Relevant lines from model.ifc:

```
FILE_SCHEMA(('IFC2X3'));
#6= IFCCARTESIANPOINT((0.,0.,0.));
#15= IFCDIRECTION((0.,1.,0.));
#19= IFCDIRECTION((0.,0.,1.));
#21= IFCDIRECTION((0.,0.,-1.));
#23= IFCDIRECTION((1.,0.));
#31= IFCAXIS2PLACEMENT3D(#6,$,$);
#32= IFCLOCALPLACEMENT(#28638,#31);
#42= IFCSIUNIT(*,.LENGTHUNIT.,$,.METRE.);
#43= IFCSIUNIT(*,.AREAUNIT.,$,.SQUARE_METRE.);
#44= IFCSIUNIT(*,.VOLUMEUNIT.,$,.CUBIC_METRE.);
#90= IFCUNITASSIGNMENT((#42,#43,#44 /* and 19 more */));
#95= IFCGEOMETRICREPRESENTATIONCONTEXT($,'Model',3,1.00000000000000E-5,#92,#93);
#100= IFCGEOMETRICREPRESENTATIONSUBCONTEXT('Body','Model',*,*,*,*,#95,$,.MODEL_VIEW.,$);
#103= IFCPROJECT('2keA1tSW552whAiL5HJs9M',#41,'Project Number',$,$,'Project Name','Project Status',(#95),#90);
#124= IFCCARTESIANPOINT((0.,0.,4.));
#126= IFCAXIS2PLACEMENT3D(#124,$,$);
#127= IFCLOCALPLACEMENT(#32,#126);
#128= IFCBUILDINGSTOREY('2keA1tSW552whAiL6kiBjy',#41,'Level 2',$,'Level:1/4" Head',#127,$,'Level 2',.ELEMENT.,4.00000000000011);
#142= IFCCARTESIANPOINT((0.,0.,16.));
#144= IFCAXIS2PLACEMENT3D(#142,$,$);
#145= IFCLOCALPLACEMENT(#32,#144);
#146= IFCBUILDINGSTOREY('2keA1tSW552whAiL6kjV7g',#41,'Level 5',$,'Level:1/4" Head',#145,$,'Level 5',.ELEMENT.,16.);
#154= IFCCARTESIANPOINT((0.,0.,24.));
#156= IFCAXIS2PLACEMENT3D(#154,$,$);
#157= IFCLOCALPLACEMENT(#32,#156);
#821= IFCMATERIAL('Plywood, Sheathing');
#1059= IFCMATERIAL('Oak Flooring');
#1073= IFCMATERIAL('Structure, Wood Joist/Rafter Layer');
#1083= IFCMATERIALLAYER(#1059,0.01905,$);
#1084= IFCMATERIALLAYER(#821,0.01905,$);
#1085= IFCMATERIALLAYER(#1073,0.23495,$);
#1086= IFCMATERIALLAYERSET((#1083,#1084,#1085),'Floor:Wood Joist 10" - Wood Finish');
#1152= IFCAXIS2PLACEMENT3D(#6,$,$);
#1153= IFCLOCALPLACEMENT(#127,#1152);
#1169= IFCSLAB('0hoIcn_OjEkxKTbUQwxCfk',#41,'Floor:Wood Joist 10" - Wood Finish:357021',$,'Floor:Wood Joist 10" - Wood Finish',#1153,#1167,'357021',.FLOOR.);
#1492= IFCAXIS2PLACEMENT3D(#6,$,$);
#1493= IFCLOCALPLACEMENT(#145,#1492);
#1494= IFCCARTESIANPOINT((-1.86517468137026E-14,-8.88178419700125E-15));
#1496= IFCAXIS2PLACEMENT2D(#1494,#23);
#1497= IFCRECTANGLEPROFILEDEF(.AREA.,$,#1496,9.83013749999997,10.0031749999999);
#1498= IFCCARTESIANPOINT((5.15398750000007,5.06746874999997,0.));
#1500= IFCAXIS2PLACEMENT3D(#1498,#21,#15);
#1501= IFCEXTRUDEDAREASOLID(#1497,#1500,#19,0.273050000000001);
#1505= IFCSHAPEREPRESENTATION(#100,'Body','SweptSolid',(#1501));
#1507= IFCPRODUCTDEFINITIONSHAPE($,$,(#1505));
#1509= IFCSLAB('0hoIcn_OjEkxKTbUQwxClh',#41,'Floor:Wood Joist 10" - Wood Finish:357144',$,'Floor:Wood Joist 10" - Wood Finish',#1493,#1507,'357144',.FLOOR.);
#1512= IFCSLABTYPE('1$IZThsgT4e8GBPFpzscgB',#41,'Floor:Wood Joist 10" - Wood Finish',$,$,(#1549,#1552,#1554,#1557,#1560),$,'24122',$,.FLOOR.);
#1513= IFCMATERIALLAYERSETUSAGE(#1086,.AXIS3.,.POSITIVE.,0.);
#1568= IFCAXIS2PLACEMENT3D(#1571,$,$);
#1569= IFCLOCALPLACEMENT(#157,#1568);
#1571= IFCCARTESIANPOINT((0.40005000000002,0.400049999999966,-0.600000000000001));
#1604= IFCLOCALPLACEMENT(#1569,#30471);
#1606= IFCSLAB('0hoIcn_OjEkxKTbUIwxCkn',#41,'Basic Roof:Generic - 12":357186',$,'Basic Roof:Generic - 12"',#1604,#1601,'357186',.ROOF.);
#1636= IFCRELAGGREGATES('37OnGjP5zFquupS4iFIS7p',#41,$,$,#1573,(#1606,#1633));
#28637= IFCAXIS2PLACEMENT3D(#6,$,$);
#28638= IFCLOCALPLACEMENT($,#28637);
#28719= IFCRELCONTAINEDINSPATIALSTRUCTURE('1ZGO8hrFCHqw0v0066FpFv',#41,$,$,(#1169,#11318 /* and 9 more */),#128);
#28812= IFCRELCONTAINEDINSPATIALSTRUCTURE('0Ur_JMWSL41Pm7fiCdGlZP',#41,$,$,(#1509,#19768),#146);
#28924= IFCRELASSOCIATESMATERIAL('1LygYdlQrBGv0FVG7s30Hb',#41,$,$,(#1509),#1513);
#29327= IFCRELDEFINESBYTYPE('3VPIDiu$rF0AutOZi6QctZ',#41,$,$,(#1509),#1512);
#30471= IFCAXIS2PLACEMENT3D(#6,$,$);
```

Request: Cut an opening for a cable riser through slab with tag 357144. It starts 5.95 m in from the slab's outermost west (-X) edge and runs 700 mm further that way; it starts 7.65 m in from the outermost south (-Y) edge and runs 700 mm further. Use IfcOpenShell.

```python
import numpy as np
import ifcopenshell
import ifcopenshell.api.feature
import ifcopenshell.api.geometry
import ifcopenshell.api.root
import ifcopenshell.geom
import ifcopenshell.util.placement
import ifcopenshell.util.representation
import ifcopenshell.util.shape
import ifcopenshell.util.unit

model = ifcopenshell.open("model.ifc")
unit_scale = ifcopenshell.util.unit.calculate_unit_scale(model)
settings = ifcopenshell.geom.settings()


def volume(element):
    """Net volume in cubic metres, openings subtracted."""
    shape = ifcopenshell.geom.create_shape(settings, element)
    return ifcopenshell.util.shape.get_volume(shape.geometry)


slab = model.by_guid("0hoIcn_OjEkxKTbUQwxClh")
before = volume(slab)

# Extent in the slab's own axes, in metres. The edges named are its -X and -Y sides.
slab_shape = ifcopenshell.geom.create_shape(settings, slab)
vertices = ifcopenshell.util.shape.get_vertices(slab_shape.geometry)
x_min, y_min, bottom = vertices.min(axis=0)
top = vertices[:, 2].max()

opening = ifcopenshell.api.root.create_entity(model, ifc_class="IfcOpeningElement", name="Cable riser opening")
context = ifcopenshell.util.representation.get_context(model, "Model", "Body", "MODEL_VIEW")
width, depth = 0.7, 0.7
outline = [(0.0, 0.0), (width, 0.0), (width, depth), (0.0, depth), (0.0, 0.0)]
# Overshoot both faces by 50 mm so the cut is clean.
shape = ifcopenshell.api.geometry.add_slab_representation(
    model, context=context, depth=top - bottom + 0.1, polyline=outline
)
ifcopenshell.api.geometry.assign_representation(model, product=opening, representation=shape)

matrix = ifcopenshell.util.placement.get_local_placement(slab.ObjectPlacement)
matrix[:, 3] = matrix @ np.append(np.array([x_min + 5.95, y_min + 7.65, bottom - 0.05]) / unit_scale, 1.0)
ifcopenshell.api.geometry.edit_object_placement(model, product=opening, matrix=matrix, is_si=False)
ifcopenshell.api.feature.add_feature(model, feature=opening, element=slab)

after = volume(slab)

print(f"slab volume {before:.3f} -> {after:.3f} m3")

model.write("model_v2.ifc")
```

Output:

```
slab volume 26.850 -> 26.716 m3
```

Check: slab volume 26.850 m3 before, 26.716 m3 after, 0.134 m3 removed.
